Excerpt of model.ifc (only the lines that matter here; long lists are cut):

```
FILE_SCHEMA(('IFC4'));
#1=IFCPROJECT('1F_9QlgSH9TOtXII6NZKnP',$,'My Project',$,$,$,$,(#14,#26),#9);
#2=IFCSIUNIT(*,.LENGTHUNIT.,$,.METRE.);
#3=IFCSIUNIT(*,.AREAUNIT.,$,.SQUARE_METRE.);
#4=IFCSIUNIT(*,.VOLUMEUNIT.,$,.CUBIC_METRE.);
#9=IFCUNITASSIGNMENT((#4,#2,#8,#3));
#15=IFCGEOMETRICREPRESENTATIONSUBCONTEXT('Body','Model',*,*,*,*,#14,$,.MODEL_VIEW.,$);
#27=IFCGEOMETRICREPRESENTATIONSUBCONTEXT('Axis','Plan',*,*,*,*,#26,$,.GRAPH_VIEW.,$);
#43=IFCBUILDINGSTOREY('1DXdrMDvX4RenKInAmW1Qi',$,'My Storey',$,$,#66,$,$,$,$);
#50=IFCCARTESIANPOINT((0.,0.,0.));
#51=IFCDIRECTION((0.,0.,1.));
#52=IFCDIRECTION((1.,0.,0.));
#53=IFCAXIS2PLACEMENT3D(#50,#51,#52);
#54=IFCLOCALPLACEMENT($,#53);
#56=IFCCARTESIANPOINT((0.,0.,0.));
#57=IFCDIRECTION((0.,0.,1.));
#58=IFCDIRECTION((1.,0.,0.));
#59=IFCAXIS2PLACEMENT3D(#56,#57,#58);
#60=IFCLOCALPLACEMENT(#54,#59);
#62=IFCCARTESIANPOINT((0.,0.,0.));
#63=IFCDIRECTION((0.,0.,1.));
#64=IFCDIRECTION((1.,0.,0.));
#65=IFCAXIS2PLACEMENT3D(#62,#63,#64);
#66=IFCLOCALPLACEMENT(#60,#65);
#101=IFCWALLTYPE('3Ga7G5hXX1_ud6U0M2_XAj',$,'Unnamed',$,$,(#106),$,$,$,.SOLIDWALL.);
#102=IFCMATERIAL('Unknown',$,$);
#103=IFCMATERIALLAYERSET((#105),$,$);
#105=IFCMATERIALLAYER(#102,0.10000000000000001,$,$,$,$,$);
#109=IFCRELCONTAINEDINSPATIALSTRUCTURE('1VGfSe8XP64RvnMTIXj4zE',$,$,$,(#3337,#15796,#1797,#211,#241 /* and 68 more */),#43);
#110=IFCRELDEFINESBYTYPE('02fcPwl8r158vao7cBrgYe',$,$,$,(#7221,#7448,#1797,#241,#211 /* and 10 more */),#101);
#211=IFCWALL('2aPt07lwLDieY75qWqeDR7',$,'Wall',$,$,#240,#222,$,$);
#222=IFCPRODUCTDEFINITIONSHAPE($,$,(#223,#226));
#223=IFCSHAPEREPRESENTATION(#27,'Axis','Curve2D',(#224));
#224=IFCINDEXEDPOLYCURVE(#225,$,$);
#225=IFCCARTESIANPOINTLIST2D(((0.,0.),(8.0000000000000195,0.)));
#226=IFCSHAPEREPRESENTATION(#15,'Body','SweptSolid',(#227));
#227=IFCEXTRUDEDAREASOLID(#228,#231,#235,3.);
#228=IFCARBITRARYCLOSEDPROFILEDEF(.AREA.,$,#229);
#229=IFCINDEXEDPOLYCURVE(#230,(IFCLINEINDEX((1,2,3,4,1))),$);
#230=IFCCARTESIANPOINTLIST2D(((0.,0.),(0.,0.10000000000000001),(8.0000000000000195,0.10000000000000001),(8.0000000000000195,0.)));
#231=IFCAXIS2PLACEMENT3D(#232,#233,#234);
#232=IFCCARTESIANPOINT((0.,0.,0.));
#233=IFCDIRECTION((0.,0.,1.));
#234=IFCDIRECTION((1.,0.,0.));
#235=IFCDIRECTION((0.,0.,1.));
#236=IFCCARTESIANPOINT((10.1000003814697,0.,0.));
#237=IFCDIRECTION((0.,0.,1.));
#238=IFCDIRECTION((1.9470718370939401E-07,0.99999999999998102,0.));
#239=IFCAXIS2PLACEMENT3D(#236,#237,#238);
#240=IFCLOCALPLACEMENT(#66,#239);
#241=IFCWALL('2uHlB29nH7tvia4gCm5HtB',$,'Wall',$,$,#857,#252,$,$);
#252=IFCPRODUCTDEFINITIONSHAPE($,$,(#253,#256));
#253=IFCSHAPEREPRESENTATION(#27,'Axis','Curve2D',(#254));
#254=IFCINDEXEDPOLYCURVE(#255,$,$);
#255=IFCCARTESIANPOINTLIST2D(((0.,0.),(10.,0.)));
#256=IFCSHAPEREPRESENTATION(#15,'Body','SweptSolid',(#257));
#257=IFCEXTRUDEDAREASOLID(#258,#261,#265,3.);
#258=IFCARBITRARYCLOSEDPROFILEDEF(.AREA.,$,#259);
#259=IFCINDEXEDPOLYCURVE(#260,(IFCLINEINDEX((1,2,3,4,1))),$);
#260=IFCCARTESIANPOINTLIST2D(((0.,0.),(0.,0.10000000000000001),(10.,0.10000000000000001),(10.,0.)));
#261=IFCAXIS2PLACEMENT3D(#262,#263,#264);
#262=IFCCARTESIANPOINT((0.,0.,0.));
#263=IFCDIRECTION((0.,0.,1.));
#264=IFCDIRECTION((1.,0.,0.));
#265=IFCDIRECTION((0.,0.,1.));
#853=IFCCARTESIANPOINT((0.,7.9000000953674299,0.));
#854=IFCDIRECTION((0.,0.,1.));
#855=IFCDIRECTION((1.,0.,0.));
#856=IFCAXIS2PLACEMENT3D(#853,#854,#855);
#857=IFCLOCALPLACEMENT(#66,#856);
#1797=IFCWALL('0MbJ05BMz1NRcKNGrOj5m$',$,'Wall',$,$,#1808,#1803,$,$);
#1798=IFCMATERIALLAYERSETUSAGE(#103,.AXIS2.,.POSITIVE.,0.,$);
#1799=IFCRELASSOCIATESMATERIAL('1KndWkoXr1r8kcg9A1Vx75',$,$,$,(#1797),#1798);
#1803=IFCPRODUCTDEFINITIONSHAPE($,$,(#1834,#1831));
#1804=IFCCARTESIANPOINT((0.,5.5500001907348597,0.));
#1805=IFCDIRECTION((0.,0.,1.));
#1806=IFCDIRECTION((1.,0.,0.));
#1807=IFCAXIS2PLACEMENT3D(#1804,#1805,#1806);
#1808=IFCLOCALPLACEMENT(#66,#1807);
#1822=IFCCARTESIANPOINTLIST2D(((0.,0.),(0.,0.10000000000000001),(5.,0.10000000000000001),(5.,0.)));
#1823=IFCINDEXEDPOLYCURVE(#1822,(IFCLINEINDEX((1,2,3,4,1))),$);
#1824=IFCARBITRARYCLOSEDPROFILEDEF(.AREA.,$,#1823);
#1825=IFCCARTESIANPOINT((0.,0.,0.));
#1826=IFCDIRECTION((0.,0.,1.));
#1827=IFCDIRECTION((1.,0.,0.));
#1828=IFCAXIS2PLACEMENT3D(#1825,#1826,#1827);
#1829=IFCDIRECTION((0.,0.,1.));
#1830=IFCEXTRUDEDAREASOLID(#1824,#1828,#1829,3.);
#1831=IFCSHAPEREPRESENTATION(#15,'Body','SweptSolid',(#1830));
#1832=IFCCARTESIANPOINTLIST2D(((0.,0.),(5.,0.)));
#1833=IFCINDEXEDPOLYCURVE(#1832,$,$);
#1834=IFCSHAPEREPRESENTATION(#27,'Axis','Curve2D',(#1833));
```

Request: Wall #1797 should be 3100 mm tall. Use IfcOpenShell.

```python
import ifcopenshell
import ifcopenshell.geom
import ifcopenshell.util.representation
import ifcopenshell.util.shape

model = ifcopenshell.open("model.ifc")
settings = ifcopenshell.geom.settings()


def volume(element):
    """Net volume in cubic metres, openings subtracted."""
    shape = ifcopenshell.geom.create_shape(settings, element)
    return ifcopenshell.util.shape.get_volume(shape.geometry)


wall = model.by_id(1797)
before = volume(wall)

body = ifcopenshell.util.representation.get_representation(wall, "Model", "Body")
solid = body.Items[0]
old_height = solid.Depth
solid.Depth = 3.1
after = volume(wall)

print(f"height {old_height:g} -> {solid.Depth:g}, volume {before:.3f} -> {after:.3f} m3")

model.write("model_edited.ifc")
```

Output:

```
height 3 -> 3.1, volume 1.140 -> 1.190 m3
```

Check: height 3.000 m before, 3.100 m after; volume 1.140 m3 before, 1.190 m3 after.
